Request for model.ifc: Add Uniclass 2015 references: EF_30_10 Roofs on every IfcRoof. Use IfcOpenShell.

First a look at what the model holds.

```python
import ifcopenshell

model = ifcopenshell.open("model.ifc")
print(model.schema)
print("classifications:", [c.Name for c in model.by_type("IfcClassification")])
for ifc_class in ("IfcDoor", "IfcRoof", "IfcStair", "IfcWall", "IfcWindow"):
    print(ifc_class, len(model.by_type(ifc_class)))
```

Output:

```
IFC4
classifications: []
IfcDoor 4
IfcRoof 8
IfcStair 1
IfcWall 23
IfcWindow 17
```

```python
import ifcopenshell
import ifcopenshell.api.classification

model = ifcopenshell.open("model.ifc")

system = ifcopenshell.api.classification.add_classification(model, classification="Uniclass 2015")

codes = {
    "IfcRoof": ("EF_30_10", "Roofs"),
}
for ifc_class, (code, name) in codes.items():
    products = model.by_type(ifc_class)
    ifcopenshell.api.classification.add_reference(
        model, products=products, classification=system, identification=code, name=name
    )
    print(code, len(products))

model.write("model-out.ifc")
```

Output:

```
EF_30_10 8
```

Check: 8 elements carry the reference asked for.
